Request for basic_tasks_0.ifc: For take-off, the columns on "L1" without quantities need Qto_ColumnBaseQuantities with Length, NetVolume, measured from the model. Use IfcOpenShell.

First a look at what the model holds.

```python
import ifcopenshell
import ifcopenshell.util.element
import ifcopenshell.util.unit

model = ifcopenshell.open("basic_tasks_0.ifc")
print(model.schema)
for unit_type in ("LENGTHUNIT", "AREAUNIT", "VOLUMEUNIT"):
    print(unit_type, ifcopenshell.util.unit.calculate_unit_scale(model, unit_type))
storey = next(s for s in model.by_type("IfcBuildingStorey") if s.Name == "L1")
columns = [e for e in ifcopenshell.util.element.get_decomposition(storey) if e.is_a("IfcColumn")]
for e in sorted(columns, key=lambda e: e.id()):
    print(e.id(), e.is_a(), e.Name, list(ifcopenshell.util.element.get_psets(e, qtos_only=True)), sep=" | ")
```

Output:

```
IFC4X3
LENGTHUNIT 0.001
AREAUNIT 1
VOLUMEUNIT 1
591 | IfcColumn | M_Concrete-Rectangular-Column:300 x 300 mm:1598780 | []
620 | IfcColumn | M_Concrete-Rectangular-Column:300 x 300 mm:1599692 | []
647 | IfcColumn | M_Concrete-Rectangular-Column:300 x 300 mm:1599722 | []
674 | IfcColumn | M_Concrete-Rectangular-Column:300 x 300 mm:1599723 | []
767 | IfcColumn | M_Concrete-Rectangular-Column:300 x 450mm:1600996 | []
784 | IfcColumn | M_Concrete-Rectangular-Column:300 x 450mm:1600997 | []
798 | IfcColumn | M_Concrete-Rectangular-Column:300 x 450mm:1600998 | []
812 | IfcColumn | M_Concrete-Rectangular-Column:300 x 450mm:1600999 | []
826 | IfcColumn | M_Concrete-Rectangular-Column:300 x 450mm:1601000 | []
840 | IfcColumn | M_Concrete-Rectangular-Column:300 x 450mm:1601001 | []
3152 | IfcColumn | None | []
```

```python
import ifcopenshell
import ifcopenshell.api.pset
import ifcopenshell.geom
import ifcopenshell.util.element
import ifcopenshell.util.shape
import ifcopenshell.util.unit

model = ifcopenshell.open("basic_tasks_0.ifc")
unit_scale = ifcopenshell.util.unit.calculate_unit_scale(model)
volume_scale = ifcopenshell.util.unit.calculate_unit_scale(model, "VOLUMEUNIT")
settings = ifcopenshell.geom.settings()

storey = next(s for s in model.by_type("IfcBuildingStorey") if s.Name == "L1")
columns = [e for e in ifcopenshell.util.element.get_decomposition(storey) if e.is_a("IfcColumn")]

for e in sorted(columns, key=lambda e: e.id()):
    if ifcopenshell.util.element.get_psets(e, qtos_only=True, should_inherit=False):
        continue
    # Geometry comes back in metres, in the element's own axes.
    shape = ifcopenshell.geom.create_shape(settings, e)
    values = {
        "Length": ifcopenshell.util.shape.get_z(shape.geometry) / unit_scale,
        "NetVolume": ifcopenshell.util.shape.get_volume(shape.geometry) / volume_scale,
    }
    qto = ifcopenshell.api.pset.add_qto(model, product=e, name="Qto_ColumnBaseQuantities")
    ifcopenshell.api.pset.edit_qto(model, qto=qto, properties=values)
    print(e.id(), {k: round(v, 3) for k, v in values.items()})

model.write("basic_tasks_0-out.ifc")
```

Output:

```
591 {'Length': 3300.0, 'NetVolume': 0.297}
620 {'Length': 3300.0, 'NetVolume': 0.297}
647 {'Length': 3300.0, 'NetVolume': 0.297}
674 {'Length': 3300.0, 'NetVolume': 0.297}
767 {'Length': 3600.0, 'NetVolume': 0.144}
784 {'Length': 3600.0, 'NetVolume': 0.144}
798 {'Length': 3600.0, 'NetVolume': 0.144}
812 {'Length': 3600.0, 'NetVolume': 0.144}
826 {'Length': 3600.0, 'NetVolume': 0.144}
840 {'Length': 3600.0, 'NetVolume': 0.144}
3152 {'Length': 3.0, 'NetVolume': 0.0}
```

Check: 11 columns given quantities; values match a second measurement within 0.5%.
